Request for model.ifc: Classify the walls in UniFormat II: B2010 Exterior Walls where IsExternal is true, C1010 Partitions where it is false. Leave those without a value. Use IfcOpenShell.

First a look at what the model holds.

```python
import ifcopenshell
import ifcopenshell.util.element

model = ifcopenshell.open("model.ifc")
print(model.schema)
print("classifications:", [c.Name for c in model.by_type("IfcClassification")])
values = [ifcopenshell.util.element.get_pset(e, "Pset_WallCommon", "IsExternal") for e in model.by_type("IfcWall")]
for value in (True, False, None):
    print("IsExternal", value, values.count(value))
```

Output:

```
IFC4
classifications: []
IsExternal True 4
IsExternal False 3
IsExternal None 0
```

```python
import ifcopenshell
import ifcopenshell.api.classification
import ifcopenshell.util.element

model = ifcopenshell.open("model.ifc")

system = ifcopenshell.api.classification.add_classification(model, classification="UniFormat II")

walls = model.by_type("IfcWall")
external = {e: ifcopenshell.util.element.get_pset(e, "Pset_WallCommon", "IsExternal") for e in walls}
for flag, code, name in ((True, "B2010", "Exterior Walls"), (False, "C1010", "Partitions")):
    products = [e for e in walls if external[e] is flag]
    ifcopenshell.api.classification.add_reference(
        model, products=products, classification=system, identification=code, name=name
    )
    print(code, len(products))

model.write("model_edited.ifc")
```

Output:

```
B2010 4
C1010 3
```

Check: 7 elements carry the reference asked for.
